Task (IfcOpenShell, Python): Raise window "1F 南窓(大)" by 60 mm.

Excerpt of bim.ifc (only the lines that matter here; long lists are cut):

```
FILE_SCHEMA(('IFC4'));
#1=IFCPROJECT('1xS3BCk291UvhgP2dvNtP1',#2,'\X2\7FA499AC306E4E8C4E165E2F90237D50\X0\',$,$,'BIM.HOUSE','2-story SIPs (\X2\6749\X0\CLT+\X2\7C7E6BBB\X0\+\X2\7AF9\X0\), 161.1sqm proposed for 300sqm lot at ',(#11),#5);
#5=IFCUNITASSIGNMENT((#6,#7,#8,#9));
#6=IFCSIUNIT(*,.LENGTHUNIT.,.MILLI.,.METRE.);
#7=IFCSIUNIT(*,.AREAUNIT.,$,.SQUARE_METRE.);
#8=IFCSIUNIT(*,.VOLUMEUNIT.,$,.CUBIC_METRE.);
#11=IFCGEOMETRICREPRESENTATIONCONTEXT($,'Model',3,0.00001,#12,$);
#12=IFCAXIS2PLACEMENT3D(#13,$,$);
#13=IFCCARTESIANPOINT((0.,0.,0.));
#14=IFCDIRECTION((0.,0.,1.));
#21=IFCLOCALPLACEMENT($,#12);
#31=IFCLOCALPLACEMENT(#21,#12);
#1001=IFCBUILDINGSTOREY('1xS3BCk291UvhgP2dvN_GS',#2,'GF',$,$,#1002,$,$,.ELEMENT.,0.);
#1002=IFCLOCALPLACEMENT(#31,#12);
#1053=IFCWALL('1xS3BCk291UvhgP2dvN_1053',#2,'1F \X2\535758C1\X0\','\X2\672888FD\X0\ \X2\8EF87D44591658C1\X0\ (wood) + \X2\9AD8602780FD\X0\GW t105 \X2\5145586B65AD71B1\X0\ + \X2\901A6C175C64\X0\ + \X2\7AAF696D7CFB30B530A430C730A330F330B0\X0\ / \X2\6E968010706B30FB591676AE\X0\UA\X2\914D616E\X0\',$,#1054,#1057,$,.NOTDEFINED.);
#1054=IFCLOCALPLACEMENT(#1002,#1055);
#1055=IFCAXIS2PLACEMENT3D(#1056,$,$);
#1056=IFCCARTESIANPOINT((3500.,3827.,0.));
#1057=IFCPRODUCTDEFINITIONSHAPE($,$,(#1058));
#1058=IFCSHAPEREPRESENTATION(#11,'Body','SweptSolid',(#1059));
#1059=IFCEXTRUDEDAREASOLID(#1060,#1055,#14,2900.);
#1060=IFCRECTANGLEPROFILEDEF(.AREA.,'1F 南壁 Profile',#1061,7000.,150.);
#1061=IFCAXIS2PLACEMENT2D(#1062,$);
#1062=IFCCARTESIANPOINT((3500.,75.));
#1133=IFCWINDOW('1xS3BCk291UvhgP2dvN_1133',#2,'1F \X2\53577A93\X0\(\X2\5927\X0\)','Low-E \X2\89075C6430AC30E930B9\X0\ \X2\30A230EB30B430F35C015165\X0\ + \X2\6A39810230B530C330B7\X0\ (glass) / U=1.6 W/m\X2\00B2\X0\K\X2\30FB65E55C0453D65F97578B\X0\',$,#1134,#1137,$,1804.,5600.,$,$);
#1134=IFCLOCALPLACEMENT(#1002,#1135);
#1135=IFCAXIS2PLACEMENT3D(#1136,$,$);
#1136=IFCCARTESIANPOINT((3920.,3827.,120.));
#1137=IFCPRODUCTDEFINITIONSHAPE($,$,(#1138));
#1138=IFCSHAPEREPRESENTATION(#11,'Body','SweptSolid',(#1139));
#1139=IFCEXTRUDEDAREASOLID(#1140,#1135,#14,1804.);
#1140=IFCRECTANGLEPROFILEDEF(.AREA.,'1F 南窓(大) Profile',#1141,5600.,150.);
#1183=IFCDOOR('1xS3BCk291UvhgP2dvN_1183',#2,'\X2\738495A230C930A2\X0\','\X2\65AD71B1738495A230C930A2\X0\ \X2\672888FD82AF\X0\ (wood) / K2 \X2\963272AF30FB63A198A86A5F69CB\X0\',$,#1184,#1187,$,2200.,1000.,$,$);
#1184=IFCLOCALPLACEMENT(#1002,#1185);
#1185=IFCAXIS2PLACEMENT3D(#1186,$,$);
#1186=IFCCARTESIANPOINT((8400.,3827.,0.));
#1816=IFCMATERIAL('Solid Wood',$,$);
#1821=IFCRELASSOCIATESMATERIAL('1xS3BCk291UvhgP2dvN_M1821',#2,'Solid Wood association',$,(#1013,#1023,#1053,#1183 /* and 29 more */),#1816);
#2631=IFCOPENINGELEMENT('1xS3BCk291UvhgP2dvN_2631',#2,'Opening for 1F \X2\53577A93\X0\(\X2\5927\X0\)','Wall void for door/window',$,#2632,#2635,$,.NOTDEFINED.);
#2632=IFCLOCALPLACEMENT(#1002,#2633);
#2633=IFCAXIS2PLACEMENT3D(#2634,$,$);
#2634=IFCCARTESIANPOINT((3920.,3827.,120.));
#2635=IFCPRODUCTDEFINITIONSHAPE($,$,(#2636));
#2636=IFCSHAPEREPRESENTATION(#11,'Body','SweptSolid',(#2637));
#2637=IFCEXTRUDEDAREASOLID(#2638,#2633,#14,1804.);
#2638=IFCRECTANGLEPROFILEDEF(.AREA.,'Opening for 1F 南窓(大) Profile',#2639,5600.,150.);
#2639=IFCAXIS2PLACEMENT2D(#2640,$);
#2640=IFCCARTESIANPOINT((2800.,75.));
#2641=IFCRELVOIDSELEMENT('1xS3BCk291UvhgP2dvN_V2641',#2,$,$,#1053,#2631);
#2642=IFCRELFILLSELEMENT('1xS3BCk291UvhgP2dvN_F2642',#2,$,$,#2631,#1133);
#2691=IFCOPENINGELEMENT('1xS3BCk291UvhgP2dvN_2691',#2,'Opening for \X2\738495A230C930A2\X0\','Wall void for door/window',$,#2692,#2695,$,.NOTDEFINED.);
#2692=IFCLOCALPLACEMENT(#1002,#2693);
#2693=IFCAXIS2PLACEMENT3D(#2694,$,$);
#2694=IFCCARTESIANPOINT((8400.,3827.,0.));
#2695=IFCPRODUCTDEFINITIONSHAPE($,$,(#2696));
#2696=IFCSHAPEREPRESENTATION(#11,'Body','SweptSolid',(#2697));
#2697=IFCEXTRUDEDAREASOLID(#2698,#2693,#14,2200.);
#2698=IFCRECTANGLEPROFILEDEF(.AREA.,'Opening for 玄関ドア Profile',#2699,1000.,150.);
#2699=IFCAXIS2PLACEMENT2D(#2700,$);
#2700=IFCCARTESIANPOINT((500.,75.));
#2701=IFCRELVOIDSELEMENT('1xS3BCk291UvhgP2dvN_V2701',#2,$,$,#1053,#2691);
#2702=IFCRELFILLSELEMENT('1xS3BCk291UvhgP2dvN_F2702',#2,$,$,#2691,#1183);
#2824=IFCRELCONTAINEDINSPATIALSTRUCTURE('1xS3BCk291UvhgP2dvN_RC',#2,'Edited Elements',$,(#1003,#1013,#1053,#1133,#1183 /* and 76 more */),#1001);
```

```python
import numpy as np
import ifcopenshell
import ifcopenshell.api.geometry
import ifcopenshell.util.placement
import ifcopenshell.util.unit

model = ifcopenshell.open("bim.ifc")
unit_scale = ifcopenshell.util.unit.calculate_unit_scale(model)

window = model.by_guid("1xS3BCk291UvhgP2dvN_1133")
opening = window.FillsVoids[0].RelatingOpeningElement
dz = 0.06 / unit_scale

shift = np.array([0.0, 0.0, dz])
# The window is not placed relative to its opening, so move both.
for product in (opening, window):
    matrix = ifcopenshell.util.placement.get_local_placement(product.ObjectPlacement)
    matrix[:3, 3] += shift
    ifcopenshell.api.geometry.edit_object_placement(model, product=product, matrix=matrix, is_si=False)

print(f"moved by {dz * unit_scale:+.3f} m")

model.write("bim_rev.ifc")
```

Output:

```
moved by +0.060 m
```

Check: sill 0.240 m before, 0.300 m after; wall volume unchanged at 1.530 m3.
